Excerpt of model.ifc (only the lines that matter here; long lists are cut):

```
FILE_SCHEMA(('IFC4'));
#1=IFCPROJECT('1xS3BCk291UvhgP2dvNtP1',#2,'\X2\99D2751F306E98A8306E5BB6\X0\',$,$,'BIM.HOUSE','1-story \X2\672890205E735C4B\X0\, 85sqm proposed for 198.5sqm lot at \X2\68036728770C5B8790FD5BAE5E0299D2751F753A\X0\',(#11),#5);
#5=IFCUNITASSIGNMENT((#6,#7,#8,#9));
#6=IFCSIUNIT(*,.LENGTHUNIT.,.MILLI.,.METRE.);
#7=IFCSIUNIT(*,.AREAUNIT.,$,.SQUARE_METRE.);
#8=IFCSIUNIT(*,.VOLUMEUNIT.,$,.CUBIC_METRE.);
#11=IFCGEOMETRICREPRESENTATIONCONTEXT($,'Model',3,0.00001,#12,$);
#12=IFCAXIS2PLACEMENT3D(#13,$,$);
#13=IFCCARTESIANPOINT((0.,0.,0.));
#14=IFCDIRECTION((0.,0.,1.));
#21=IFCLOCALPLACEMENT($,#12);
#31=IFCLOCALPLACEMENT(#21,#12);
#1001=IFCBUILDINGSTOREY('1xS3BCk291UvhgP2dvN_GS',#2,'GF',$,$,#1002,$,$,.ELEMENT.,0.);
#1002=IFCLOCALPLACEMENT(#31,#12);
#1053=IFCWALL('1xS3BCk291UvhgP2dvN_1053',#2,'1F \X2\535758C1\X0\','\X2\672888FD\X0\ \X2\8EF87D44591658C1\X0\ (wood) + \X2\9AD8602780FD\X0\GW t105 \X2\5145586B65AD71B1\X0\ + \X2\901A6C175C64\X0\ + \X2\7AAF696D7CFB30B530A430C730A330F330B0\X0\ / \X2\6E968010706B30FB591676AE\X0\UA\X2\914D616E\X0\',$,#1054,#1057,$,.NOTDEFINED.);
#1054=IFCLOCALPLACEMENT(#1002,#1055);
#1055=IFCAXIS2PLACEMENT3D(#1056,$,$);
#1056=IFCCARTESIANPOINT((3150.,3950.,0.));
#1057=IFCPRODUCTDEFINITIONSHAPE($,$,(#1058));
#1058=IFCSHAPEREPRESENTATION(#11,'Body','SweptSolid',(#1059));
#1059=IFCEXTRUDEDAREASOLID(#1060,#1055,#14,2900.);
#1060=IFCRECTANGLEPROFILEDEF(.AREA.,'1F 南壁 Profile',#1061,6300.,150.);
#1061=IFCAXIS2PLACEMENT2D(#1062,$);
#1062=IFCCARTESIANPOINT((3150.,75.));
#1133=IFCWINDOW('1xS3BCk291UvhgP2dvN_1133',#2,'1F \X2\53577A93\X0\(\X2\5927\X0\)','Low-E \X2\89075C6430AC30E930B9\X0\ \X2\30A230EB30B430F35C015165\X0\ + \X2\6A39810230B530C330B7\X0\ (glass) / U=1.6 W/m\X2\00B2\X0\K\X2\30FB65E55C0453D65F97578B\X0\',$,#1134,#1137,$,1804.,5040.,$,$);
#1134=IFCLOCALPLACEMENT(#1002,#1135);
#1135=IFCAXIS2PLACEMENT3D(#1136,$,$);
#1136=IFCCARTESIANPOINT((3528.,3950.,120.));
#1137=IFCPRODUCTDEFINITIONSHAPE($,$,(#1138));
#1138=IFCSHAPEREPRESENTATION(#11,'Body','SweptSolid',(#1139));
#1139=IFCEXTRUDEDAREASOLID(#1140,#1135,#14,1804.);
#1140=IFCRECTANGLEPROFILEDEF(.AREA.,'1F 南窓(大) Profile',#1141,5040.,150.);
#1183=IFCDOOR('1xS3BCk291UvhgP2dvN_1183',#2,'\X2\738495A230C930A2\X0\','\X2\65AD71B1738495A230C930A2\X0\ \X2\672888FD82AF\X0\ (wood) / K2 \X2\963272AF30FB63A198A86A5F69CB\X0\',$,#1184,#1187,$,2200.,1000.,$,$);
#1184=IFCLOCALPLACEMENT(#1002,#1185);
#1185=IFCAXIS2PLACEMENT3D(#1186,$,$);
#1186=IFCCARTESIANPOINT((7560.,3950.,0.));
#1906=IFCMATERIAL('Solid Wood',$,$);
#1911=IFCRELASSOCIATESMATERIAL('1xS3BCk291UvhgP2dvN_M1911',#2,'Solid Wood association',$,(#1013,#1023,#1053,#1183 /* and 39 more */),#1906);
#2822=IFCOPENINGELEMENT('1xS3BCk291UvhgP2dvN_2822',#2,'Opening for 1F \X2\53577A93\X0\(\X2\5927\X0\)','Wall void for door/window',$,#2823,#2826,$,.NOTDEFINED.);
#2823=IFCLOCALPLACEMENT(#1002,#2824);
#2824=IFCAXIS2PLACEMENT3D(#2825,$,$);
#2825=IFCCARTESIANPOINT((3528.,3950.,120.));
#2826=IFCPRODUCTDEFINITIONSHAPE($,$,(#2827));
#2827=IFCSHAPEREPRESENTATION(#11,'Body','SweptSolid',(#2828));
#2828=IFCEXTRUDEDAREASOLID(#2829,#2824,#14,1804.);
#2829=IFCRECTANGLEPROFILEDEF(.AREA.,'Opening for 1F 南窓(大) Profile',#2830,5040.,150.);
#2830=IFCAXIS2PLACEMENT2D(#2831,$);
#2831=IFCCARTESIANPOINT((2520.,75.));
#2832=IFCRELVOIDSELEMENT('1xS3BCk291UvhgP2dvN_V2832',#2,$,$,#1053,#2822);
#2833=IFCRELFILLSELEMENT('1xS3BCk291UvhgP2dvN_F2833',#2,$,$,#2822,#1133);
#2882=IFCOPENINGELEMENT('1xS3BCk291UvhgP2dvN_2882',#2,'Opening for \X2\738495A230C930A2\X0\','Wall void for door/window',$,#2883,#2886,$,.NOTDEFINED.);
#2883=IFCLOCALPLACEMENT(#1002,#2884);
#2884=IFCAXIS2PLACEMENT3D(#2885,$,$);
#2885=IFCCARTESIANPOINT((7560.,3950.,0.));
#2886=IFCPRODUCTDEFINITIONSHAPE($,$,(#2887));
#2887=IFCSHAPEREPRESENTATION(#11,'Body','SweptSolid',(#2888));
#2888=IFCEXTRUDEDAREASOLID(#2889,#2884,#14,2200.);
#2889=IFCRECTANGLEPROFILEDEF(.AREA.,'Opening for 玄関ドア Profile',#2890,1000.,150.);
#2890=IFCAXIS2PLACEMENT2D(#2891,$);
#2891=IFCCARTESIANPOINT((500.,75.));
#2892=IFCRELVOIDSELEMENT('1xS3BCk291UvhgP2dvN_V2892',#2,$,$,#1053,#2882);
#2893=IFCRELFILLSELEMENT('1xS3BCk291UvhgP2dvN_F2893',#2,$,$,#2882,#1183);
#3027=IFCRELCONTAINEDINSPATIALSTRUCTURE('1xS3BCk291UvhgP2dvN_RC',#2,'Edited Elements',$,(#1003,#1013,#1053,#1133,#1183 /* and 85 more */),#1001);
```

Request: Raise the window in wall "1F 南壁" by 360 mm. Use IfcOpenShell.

```python
import numpy as np
import ifcopenshell
import ifcopenshell.api.geometry
import ifcopenshell.util.placement
import ifcopenshell.util.unit

model = ifcopenshell.open("model.ifc")
unit_scale = ifcopenshell.util.unit.calculate_unit_scale(model)

window = model.by_guid("1xS3BCk291UvhgP2dvN_1133")
opening = window.FillsVoids[0].RelatingOpeningElement
dz = 0.36 / unit_scale

shift = np.array([0.0, 0.0, dz])
# The window is not placed relative to its opening, so move both.
for product in (opening, window):
    matrix = ifcopenshell.util.placement.get_local_placement(product.ObjectPlacement)
    matrix[:3, 3] += shift
    ifcopenshell.api.geometry.edit_object_placement(model, product=product, matrix=matrix, is_si=False)

print(f"moved by {dz * unit_scale:+.3f} m")

model.write("model_rev.ifc")
```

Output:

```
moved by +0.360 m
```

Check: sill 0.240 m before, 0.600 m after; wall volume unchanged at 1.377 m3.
